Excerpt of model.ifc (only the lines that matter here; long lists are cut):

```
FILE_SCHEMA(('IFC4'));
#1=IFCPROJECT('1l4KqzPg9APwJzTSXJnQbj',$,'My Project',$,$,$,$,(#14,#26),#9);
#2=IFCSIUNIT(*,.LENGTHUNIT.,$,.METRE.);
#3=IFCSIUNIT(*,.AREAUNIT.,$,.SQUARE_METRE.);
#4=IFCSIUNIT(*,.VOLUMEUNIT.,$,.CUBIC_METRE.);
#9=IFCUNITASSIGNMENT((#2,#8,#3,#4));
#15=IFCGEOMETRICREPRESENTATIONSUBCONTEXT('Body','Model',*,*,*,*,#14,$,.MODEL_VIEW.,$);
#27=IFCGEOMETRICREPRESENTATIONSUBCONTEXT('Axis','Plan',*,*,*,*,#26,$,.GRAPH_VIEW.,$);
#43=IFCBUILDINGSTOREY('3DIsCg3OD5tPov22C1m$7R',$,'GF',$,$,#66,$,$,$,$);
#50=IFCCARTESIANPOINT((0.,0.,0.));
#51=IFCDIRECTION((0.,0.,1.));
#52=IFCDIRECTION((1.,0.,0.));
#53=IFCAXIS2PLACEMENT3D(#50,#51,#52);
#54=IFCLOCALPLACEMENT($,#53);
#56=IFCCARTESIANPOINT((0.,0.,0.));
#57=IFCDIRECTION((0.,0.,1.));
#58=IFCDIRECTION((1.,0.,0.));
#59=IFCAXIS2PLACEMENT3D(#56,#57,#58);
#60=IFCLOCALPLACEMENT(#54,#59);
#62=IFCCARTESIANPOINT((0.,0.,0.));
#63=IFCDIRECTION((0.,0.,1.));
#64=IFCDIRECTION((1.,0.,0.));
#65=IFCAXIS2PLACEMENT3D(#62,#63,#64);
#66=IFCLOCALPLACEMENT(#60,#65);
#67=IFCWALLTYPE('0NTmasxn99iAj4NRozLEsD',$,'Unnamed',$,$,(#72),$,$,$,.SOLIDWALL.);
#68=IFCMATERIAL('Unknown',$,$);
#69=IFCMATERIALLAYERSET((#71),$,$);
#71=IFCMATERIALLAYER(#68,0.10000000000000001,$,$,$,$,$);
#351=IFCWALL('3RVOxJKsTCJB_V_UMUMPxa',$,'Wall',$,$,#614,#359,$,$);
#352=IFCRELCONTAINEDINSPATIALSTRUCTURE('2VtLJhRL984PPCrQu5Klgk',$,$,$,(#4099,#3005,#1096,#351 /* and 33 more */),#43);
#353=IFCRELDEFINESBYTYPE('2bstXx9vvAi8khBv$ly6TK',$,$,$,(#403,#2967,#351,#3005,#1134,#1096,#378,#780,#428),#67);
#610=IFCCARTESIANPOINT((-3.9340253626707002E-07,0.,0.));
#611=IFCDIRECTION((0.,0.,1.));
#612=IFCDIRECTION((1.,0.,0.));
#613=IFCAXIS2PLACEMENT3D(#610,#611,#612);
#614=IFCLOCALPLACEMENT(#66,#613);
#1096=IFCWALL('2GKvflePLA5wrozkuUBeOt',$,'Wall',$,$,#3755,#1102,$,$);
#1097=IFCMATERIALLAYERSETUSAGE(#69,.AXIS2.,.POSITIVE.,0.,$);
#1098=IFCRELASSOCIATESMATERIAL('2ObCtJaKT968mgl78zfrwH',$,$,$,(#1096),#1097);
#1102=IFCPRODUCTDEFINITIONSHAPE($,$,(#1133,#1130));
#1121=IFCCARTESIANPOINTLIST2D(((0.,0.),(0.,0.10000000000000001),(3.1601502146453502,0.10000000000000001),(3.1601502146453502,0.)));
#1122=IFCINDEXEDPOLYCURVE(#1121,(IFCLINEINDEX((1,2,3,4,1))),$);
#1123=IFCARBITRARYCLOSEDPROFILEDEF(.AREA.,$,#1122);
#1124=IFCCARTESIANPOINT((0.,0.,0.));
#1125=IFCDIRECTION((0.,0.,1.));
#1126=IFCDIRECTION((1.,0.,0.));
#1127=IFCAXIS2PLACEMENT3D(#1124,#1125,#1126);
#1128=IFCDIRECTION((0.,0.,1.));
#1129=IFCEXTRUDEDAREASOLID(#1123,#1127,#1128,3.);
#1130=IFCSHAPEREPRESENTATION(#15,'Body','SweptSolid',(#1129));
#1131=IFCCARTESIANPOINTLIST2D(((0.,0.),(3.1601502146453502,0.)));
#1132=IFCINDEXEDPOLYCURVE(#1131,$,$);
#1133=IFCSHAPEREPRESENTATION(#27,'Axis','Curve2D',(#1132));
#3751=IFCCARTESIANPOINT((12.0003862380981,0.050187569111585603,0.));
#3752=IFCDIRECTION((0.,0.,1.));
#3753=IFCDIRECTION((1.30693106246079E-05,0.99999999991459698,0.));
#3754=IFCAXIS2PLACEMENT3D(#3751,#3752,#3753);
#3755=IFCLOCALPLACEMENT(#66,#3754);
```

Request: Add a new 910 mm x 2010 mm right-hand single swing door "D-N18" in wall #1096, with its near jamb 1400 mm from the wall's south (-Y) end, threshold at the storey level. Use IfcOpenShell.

```python
import numpy as np
import ifcopenshell
import ifcopenshell.api.feature
import ifcopenshell.api.geometry
import ifcopenshell.api.root
import ifcopenshell.api.spatial
import ifcopenshell.geom
import ifcopenshell.util.element
import ifcopenshell.util.placement
import ifcopenshell.util.representation
import ifcopenshell.util.shape
import ifcopenshell.util.unit

model = ifcopenshell.open("model.ifc")
unit_scale = ifcopenshell.util.unit.calculate_unit_scale(model)
settings = ifcopenshell.geom.settings()


def volume(element):
    """Net volume in cubic metres, openings subtracted."""
    shape = ifcopenshell.geom.create_shape(settings, element)
    return ifcopenshell.util.shape.get_volume(shape.geometry)


wall = model.by_guid("2GKvflePLA5wrozkuUBeOt")
storey = ifcopenshell.util.element.get_container(wall, ifc_class="IfcBuildingStorey")
context = ifcopenshell.util.representation.get_context(model, "Model", "Body", "MODEL_VIEW")
before = volume(wall)

width, height, from_end, sill = 0.91, 2.01, 1.4, 0.0  # metres

# The wall runs along its own X axis, and the end named is its -X end.
wall_shape = ifcopenshell.geom.create_shape(settings, wall)
x, y, z = ifcopenshell.util.shape.get_vertices(wall_shape.geometry).T
start = x.min() + from_end
face, thickness = float(y.min()), float(y.max() - y.min())
wall_matrix = ifcopenshell.util.placement.get_local_placement(wall.ObjectPlacement)
level = ifcopenshell.util.placement.get_local_placement(storey.ObjectPlacement)[2, 3]


def in_wall(x, y):
    """Placement at x, y metres in the wall's axes, at sill height."""
    matrix = wall_matrix.copy()
    matrix[:, 3] = wall_matrix @ np.array([x / unit_scale, y / unit_scale, 0.0, 1.0])
    matrix[2, 3] = level + sill / unit_scale
    return matrix


# Opening: a box that overshoots both wall faces by 50 mm.
opening = ifcopenshell.api.root.create_entity(model, ifc_class="IfcOpeningElement", predefined_type="OPENING")
box = ifcopenshell.api.geometry.add_wall_representation(
    model, context=context, length=width, height=height, thickness=thickness + 0.1
)
ifcopenshell.api.geometry.assign_representation(model, product=opening, representation=box)
ifcopenshell.api.geometry.edit_object_placement(model, product=opening, matrix=in_wall(start, face - 0.05), is_si=False)
ifcopenshell.api.feature.add_feature(model, feature=opening, element=wall)

door = ifcopenshell.api.root.create_entity(model, ifc_class="IfcDoor", name="D-N18", predefined_type="DOOR")
door.OverallWidth, door.OverallHeight = width / unit_scale, height / unit_scale
door.OperationType = "SINGLE_SWING_RIGHT"
body = ifcopenshell.api.geometry.add_door_representation(
    model,
    context=context,
    overall_width=door.OverallWidth,
    overall_height=door.OverallHeight,
    operation_type="SINGLE_SWING_RIGHT",
    lining_properties={"LiningDepth": thickness / unit_scale, "ThresholdDepth": thickness / unit_scale},
)
ifcopenshell.api.geometry.assign_representation(model, product=door, representation=body)
ifcopenshell.api.spatial.assign_container(model, products=[door], relating_structure=storey)
ifcopenshell.api.feature.add_filling(model, opening=opening, element=door)

# The lining spans the wall, so the door starts at the wall face.
ifcopenshell.api.geometry.edit_object_placement(model, product=door, matrix=in_wall(start, face), is_si=False)

after = volume(wall)

print(f"wall volume {before:.3f} -> {after:.3f} m3")

model.write("model_v2.ifc")
```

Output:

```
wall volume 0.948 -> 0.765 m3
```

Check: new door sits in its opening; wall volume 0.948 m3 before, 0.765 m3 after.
